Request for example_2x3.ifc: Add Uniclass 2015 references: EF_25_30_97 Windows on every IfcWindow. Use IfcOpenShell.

First a look at what the model holds.

```python
import ifcopenshell

model = ifcopenshell.open("example_2x3.ifc")
print(model.schema)
print("classifications:", [c.Name for c in model.by_type("IfcClassification")])
for ifc_class in ("IfcDoor", "IfcRoof", "IfcStair", "IfcWall", "IfcWindow"):
    print(ifc_class, len(model.by_type(ifc_class)))
```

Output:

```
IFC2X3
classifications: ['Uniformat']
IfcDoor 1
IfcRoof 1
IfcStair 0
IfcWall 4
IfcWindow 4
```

```python
import ifcopenshell
import ifcopenshell.api.classification

model = ifcopenshell.open("example_2x3.ifc")

# IFC2X3 requires Source and Edition and has no link from the project to the system.
system = model.create_entity("IfcClassification", Source="NBS", Edition="2015", Name="Uniclass 2015")

codes = {
    "IfcWindow": ("EF_25_30_97", "Windows"),
}
for ifc_class, (code, name) in codes.items():
    products = model.by_type(ifc_class)
    ifcopenshell.api.classification.add_reference(
        model, products=products, classification=system, identification=code, name=name
    )
    print(code, len(products))

model.write("example_2x3_v2.ifc")
```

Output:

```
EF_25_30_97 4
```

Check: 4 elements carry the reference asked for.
